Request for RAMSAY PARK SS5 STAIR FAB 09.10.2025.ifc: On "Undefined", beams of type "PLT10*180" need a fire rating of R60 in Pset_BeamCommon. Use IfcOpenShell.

First a look at what the model holds.

```python
import ifcopenshell
import ifcopenshell.util.element

model = ifcopenshell.open("RAMSAY PARK SS5 STAIR FAB 09.10.2025.ifc")
print(model.schema)
storey = next(s for s in model.by_type("IfcBuildingStorey") if s.Name == "Undefined")
beams = [e for e in ifcopenshell.util.element.get_decomposition(storey) if e.is_a("IfcBeam")]
seen = {}
for e in beams:
    element_type = ifcopenshell.util.element.get_type(e)
    key = (element_type.Name if element_type != e and element_type else None, ifcopenshell.util.element.get_pset(e, "Pset_BeamCommon", "FireRating"))
    seen[key] = seen.get(key, 0) + 1
for (name, value), count in sorted(seen.items(), key=str):
    print(count, "x", name, "|", value)
```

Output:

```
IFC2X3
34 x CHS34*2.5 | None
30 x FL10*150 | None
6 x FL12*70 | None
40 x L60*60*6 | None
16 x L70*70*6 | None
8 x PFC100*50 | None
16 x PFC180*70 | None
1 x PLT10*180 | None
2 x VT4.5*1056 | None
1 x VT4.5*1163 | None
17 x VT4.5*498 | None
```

```python
import ifcopenshell
import ifcopenshell.api.pset
import ifcopenshell.util.element

model = ifcopenshell.open("RAMSAY PARK SS5 STAIR FAB 09.10.2025.ifc")

storey = next(s for s in model.by_type("IfcBuildingStorey") if s.Name == "Undefined")
beams = [e for e in ifcopenshell.util.element.get_decomposition(storey) if e.is_a("IfcBeam")]

count = 0
for e in beams:
    element_type = ifcopenshell.util.element.get_type(e)
    if element_type in (None, e) or element_type.Name != "PLT10*180":
        continue
    # add_pset returns the element's existing set when there is one.
    pset = ifcopenshell.api.pset.add_pset(model, product=e, name="Pset_BeamCommon")
    ifcopenshell.api.pset.edit_pset(model, pset=pset, properties={"FireRating": "R60"})
    count += 1

print(count, "beams updated")

model.write("RAMSAY PARK SS5 STAIR FAB 09.10.2025_v2.ifc")
```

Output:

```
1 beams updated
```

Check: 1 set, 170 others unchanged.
